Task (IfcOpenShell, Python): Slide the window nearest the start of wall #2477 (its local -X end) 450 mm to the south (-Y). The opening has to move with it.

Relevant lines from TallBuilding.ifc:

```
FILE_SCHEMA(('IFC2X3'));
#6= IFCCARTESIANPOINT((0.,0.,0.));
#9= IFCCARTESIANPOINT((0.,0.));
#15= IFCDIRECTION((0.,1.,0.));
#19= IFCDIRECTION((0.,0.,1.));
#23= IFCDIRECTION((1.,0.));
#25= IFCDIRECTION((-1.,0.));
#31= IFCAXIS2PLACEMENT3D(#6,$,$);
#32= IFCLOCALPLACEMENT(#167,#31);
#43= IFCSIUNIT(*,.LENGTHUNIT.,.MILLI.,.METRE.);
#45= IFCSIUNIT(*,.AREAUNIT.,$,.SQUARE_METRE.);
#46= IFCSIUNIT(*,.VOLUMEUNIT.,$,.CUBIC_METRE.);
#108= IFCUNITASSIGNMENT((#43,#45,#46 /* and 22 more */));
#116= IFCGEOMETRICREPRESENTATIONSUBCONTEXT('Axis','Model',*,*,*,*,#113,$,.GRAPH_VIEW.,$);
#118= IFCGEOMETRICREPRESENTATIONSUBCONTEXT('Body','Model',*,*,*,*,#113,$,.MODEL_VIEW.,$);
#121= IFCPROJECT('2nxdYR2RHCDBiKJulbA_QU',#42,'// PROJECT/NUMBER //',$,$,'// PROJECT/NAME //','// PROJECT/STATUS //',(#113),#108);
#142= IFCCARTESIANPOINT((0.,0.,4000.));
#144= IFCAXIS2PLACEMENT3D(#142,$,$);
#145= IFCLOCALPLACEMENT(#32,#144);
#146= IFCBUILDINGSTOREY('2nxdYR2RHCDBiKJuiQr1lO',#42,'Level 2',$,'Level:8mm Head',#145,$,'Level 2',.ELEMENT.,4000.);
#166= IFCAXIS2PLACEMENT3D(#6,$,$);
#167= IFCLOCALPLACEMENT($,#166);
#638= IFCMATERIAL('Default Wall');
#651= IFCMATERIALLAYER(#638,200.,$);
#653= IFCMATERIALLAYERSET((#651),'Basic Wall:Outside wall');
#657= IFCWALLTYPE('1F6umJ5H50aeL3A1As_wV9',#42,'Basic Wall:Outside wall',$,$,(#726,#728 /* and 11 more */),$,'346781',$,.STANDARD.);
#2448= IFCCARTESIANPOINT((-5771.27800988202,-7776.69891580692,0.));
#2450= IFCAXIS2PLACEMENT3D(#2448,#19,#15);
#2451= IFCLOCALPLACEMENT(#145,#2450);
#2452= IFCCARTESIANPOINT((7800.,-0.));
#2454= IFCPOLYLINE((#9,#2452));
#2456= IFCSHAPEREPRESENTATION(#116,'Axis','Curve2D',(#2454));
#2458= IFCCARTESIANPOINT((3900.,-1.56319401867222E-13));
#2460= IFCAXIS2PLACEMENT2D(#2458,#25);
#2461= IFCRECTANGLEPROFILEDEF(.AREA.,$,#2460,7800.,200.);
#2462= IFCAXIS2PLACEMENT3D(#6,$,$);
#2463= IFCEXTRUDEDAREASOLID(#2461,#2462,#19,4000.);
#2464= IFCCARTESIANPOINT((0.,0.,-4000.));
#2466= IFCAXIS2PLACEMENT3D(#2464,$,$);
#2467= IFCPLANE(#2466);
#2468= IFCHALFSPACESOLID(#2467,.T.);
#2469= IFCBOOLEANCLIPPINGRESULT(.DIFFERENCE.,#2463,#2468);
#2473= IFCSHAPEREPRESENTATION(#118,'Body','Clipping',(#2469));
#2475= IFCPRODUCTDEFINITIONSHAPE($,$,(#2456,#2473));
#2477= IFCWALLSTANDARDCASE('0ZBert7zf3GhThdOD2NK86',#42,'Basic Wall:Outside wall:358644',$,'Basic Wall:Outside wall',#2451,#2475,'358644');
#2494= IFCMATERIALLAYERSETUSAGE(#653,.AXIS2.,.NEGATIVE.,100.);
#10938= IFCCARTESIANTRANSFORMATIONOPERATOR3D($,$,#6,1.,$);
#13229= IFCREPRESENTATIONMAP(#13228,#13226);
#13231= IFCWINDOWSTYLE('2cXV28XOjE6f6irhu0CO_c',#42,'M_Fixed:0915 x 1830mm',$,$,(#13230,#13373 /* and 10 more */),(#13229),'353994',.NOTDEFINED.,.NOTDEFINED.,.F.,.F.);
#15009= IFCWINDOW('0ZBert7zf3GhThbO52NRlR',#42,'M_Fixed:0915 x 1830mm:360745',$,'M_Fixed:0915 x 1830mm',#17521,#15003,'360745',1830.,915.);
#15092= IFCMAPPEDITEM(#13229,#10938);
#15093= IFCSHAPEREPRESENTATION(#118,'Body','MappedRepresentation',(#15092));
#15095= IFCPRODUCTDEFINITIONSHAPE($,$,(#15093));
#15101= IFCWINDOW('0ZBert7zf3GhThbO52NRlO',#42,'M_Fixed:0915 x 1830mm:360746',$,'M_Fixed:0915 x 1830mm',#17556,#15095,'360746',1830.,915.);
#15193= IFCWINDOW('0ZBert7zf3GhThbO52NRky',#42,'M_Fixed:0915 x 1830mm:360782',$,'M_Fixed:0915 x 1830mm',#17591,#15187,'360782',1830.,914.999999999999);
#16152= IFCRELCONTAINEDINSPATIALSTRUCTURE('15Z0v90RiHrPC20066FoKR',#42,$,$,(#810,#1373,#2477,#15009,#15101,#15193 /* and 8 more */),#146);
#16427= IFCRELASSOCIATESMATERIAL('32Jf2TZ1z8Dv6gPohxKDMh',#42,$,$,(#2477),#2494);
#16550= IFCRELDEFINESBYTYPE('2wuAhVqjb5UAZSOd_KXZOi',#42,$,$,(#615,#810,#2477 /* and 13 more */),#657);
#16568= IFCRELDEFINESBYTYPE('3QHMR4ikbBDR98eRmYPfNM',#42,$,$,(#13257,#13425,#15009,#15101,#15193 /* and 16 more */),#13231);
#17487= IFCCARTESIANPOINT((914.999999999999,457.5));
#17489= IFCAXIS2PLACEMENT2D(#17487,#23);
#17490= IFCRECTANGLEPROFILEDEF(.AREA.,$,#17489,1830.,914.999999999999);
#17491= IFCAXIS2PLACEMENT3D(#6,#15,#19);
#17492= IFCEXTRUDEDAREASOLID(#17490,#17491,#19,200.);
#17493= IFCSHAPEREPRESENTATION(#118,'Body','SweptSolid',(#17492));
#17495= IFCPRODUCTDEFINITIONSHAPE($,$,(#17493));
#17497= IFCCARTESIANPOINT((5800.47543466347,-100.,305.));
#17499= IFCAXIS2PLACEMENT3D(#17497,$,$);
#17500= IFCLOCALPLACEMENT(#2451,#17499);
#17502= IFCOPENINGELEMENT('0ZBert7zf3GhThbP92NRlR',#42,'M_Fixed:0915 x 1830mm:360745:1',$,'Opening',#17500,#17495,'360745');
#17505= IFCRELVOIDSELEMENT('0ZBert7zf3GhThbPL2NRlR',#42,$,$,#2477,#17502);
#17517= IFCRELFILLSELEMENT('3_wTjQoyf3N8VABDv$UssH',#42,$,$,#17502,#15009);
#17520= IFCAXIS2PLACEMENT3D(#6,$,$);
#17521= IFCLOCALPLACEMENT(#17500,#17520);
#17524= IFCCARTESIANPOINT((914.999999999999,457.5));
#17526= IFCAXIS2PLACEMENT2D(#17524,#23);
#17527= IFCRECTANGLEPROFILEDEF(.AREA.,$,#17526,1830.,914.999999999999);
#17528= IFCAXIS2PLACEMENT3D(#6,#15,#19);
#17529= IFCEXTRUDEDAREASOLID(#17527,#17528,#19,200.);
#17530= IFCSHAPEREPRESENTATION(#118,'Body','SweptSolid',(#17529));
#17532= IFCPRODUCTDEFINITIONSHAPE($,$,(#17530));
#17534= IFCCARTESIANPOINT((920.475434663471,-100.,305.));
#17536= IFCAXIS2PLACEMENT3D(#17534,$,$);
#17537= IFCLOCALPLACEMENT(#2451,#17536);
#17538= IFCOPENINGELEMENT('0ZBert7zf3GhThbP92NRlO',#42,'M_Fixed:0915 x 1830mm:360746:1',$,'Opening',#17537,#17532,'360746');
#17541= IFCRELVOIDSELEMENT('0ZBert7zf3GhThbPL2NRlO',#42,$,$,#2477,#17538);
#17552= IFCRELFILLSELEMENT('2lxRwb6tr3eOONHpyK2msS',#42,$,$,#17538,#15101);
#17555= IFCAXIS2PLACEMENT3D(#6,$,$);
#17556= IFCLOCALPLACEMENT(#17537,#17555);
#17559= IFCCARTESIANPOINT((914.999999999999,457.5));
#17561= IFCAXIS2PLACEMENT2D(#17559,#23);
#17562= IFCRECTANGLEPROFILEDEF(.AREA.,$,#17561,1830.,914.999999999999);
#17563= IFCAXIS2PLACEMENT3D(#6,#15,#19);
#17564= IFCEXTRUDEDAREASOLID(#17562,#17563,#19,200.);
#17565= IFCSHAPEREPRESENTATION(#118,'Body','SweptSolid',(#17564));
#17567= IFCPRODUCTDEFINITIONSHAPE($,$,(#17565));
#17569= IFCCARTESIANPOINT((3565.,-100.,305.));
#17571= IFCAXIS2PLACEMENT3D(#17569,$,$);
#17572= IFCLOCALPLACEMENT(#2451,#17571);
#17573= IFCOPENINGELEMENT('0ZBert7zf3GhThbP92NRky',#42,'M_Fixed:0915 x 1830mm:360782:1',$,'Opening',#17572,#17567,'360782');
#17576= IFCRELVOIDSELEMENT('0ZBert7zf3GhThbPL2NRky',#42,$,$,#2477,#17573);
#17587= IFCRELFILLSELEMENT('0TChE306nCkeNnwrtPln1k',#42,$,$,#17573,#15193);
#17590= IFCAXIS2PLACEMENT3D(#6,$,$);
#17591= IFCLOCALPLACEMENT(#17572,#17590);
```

```python
import ifcopenshell
import ifcopenshell.api.geometry
import ifcopenshell.util.placement
import ifcopenshell.util.unit

model = ifcopenshell.open("TallBuilding.ifc")
unit_scale = ifcopenshell.util.unit.calculate_unit_scale(model)

window = model.by_guid("0ZBert7zf3GhThbO52NRlO")
opening = window.FillsVoids[0].RelatingOpeningElement
wall = opening.VoidsElements[0].RelatingBuildingElement

wall_matrix = ifcopenshell.util.placement.get_local_placement(wall.ObjectPlacement)
shift = wall_matrix[:3, 0] * -0.45 / unit_scale
before = ifcopenshell.util.placement.get_local_placement(window.ObjectPlacement)[:3, 3].copy()

# The window is placed relative to its opening, so it follows when the opening moves.
matrix = ifcopenshell.util.placement.get_local_placement(opening.ObjectPlacement)
matrix[:3, 3] += shift
ifcopenshell.api.geometry.edit_object_placement(
    model, product=opening, matrix=matrix, is_si=False, should_transform_children=True
)

after = ifcopenshell.util.placement.get_local_placement(window.ObjectPlacement)[:3, 3]
print("window moved by", (after - before).round(3) + 0.0)

model.write("TallBuilding_updated.ifc")
```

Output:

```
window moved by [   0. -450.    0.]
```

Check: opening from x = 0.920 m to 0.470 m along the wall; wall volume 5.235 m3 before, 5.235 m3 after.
